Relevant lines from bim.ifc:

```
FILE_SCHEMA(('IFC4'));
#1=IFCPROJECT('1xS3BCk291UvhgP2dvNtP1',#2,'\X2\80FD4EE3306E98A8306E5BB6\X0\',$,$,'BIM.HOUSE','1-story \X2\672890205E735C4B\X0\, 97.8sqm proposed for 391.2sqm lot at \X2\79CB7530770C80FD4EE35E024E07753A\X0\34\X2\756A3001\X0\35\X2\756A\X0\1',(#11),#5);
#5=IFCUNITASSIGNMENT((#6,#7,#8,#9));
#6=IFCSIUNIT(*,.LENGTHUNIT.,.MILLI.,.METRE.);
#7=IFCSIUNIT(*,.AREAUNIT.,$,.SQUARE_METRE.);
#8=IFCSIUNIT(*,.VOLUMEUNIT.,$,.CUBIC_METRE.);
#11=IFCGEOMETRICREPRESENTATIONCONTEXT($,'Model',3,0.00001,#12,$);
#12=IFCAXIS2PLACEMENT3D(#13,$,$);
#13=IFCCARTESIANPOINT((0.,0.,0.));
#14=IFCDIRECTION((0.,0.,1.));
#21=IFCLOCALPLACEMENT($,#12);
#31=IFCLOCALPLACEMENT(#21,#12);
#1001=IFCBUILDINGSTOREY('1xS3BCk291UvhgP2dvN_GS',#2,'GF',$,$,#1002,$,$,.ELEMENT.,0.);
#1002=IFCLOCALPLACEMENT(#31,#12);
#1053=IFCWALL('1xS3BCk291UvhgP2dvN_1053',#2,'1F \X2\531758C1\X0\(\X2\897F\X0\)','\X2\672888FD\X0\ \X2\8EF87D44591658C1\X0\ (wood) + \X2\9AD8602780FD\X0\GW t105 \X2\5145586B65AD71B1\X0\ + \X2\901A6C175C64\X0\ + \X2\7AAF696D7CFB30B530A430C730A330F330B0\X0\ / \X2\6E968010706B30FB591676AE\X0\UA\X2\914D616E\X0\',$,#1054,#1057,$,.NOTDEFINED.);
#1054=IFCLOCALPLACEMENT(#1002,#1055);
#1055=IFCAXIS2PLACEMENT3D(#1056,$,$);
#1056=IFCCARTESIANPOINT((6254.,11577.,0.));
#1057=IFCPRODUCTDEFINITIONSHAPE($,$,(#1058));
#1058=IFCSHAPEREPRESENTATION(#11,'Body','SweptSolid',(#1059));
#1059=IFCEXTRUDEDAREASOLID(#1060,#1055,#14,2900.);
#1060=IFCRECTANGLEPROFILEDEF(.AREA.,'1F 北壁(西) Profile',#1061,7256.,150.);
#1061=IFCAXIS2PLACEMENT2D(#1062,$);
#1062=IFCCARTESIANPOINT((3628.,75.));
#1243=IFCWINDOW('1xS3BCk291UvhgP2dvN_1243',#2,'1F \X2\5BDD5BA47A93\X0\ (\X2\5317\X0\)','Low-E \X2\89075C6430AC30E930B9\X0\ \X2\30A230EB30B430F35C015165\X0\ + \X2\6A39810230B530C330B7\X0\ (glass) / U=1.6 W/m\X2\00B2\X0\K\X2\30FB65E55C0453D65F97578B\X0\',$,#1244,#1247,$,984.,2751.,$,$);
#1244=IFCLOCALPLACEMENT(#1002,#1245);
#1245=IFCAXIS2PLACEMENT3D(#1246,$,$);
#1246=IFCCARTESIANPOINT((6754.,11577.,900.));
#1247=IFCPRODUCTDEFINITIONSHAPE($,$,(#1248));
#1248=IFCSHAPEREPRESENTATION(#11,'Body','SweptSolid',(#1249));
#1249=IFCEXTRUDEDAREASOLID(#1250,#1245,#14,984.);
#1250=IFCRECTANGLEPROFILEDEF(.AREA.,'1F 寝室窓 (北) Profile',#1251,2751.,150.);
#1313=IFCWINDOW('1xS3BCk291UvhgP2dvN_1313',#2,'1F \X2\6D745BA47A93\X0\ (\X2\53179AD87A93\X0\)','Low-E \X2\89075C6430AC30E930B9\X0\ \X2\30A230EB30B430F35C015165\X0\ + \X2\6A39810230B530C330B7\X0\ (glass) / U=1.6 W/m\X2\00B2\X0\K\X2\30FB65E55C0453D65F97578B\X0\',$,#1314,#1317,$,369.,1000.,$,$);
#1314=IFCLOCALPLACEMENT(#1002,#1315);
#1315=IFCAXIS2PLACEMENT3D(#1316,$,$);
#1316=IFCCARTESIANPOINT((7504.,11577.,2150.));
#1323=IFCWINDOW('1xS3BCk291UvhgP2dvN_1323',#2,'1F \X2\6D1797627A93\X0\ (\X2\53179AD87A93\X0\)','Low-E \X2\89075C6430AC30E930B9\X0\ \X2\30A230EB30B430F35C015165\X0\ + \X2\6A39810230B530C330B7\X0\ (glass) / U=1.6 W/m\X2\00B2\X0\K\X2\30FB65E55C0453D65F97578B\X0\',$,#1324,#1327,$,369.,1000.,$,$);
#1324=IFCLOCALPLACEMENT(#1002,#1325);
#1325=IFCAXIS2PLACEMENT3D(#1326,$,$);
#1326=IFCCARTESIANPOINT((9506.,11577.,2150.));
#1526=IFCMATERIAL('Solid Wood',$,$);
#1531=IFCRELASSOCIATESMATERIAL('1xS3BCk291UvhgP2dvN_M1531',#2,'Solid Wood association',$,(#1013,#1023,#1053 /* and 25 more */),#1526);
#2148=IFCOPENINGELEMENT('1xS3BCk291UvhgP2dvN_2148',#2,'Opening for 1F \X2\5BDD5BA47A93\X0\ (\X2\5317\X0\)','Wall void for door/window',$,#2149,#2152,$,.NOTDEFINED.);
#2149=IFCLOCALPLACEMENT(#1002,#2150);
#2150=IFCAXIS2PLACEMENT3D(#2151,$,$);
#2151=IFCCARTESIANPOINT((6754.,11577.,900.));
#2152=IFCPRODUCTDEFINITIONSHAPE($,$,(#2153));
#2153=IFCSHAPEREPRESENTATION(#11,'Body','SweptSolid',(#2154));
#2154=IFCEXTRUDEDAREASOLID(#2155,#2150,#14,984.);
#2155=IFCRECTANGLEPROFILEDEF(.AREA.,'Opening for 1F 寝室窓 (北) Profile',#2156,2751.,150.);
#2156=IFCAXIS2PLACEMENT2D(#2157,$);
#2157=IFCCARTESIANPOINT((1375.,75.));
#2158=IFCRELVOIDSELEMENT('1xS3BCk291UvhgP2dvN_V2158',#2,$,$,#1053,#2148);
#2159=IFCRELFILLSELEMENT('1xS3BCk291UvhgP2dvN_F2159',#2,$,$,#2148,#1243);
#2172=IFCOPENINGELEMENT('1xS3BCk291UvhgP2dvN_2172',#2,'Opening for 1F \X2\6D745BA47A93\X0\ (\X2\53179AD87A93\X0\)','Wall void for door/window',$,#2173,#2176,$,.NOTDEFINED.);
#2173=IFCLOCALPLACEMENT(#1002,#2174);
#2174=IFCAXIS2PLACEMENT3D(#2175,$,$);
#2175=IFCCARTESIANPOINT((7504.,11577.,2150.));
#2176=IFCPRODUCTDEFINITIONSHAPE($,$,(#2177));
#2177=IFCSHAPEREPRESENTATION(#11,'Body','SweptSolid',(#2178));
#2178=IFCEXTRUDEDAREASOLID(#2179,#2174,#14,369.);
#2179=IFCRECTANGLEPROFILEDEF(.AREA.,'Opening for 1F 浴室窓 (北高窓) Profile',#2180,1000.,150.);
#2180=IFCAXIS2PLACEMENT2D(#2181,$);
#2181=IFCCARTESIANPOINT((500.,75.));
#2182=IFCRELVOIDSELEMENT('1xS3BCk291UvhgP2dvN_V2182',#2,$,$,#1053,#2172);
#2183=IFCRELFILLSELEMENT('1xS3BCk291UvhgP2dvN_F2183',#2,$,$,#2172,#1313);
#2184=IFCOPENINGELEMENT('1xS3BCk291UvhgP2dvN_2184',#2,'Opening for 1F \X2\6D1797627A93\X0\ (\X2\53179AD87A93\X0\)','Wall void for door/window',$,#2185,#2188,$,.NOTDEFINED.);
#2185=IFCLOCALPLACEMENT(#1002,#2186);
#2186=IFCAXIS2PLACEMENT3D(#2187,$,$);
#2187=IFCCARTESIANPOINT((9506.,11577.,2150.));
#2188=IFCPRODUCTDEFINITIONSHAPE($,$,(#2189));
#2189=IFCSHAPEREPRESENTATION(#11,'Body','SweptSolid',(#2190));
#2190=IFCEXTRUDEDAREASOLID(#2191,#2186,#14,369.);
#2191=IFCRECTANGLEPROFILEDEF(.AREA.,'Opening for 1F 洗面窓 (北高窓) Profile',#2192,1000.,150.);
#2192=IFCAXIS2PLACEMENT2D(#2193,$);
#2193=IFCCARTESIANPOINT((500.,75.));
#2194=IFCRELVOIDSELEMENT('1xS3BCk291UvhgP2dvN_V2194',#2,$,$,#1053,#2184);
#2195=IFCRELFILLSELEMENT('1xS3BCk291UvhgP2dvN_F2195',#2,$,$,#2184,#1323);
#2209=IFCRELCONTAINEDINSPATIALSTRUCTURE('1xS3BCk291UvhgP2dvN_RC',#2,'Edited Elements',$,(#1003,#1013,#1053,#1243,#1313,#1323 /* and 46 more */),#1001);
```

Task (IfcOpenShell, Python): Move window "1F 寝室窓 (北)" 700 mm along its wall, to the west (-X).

```python
import ifcopenshell
import ifcopenshell.api.geometry
import ifcopenshell.util.placement
import ifcopenshell.util.unit

model = ifcopenshell.open("bim.ifc")
unit_scale = ifcopenshell.util.unit.calculate_unit_scale(model)

window = model.by_guid("1xS3BCk291UvhgP2dvN_1243")
opening = window.FillsVoids[0].RelatingOpeningElement
wall = opening.VoidsElements[0].RelatingBuildingElement

wall_matrix = ifcopenshell.util.placement.get_local_placement(wall.ObjectPlacement)
shift = wall_matrix[:3, 0] * -0.7 / unit_scale
before = ifcopenshell.util.placement.get_local_placement(window.ObjectPlacement)[:3, 3].copy()

# The window is not placed relative to its opening, so move both.
for product in (opening, window):
    matrix = ifcopenshell.util.placement.get_local_placement(product.ObjectPlacement)
    matrix[:3, 3] += shift
    ifcopenshell.api.geometry.edit_object_placement(model, product=product, matrix=matrix, is_si=False)

after = ifcopenshell.util.placement.get_local_placement(window.ObjectPlacement)[:3, 3]
print("window moved by", (after - before).round(3) + 0.0)

model.write("bim-out.ifc")
```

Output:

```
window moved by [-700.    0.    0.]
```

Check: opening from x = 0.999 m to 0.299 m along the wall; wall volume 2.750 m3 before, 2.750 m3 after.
